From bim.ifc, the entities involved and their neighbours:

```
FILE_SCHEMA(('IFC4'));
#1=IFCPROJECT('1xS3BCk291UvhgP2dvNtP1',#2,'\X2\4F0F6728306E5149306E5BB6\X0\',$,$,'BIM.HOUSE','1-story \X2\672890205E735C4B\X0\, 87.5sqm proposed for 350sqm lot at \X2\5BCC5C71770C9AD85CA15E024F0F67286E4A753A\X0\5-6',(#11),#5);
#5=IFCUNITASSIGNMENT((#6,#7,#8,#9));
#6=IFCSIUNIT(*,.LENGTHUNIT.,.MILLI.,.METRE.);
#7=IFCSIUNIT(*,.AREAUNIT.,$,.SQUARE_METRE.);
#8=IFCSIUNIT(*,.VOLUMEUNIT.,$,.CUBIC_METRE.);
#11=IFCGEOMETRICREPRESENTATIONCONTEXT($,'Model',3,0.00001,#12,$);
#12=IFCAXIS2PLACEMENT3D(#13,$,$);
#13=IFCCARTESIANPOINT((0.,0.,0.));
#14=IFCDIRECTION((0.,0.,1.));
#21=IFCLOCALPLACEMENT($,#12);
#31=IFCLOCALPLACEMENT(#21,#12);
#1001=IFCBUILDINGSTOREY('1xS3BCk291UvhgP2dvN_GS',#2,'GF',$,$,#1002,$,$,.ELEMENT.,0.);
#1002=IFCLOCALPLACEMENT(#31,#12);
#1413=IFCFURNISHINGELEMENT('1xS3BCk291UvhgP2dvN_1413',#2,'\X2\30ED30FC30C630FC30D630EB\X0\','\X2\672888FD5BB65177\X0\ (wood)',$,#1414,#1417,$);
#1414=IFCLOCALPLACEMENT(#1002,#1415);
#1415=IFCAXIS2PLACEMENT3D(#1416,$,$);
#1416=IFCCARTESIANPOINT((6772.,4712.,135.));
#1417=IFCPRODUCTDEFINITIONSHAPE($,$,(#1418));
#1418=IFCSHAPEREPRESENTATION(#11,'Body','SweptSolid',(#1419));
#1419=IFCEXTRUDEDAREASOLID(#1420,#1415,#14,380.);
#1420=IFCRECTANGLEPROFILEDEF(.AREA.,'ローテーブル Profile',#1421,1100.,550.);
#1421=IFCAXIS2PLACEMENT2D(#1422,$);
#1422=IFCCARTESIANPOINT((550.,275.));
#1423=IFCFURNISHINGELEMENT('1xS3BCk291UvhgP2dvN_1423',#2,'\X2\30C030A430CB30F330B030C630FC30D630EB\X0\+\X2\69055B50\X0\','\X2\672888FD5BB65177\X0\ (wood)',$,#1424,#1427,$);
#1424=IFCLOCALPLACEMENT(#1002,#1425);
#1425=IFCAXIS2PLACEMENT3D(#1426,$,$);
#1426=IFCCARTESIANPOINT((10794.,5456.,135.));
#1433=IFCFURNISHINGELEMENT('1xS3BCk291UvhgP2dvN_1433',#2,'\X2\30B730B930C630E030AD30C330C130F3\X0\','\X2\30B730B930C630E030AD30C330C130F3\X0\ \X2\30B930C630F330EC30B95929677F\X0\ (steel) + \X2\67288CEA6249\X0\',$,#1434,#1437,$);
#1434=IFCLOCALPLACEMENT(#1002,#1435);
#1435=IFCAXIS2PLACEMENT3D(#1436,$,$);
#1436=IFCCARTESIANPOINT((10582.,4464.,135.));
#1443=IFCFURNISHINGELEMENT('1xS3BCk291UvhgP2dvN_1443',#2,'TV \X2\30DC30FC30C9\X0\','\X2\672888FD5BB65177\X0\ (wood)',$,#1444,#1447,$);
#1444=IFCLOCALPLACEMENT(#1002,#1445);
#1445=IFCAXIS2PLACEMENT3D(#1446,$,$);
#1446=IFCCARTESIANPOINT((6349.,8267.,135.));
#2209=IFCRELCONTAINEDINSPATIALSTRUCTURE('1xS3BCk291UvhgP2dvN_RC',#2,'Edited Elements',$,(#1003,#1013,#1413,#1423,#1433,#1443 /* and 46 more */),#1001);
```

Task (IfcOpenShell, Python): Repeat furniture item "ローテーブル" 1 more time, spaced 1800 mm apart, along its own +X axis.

```python
import ifcopenshell
import ifcopenshell.api.geometry
import ifcopenshell.api.root
import ifcopenshell.util.element
import ifcopenshell.util.placement
import ifcopenshell.util.unit

model = ifcopenshell.open("bim.ifc")
unit_scale = ifcopenshell.util.unit.calculate_unit_scale(model)


def reuse_history(source, copy):
    """copy_class also copies each property set's owner history, people and application; keep the originals."""
    for rel in copy.IsDefinedBy:
        if rel.is_a("IfcRelDefinesByProperties") and (history := rel.RelatingPropertyDefinition.OwnerHistory):
            rel.RelatingPropertyDefinition.OwnerHistory = source.OwnerHistory
            ifcopenshell.util.element.remove_deep2(model, history)


source = model.by_guid("1xS3BCk291UvhgP2dvN_1413")
base = ifcopenshell.util.placement.get_local_placement(source.ObjectPlacement)
step = base[:3, 0] * 1.8 / unit_scale

for i in range(1, 2):
    copy = ifcopenshell.api.root.copy_class(model, product=source)
    copy.Representation = ifcopenshell.util.element.copy_deep(
        model, source.Representation, exclude=["IfcGeometricRepresentationContext", "IfcRepresentationMap"]
    )
    reuse_history(source, copy)
    matrix = base.copy()
    matrix[:3, 3] += i * step
    print("added at", matrix[:3, 3].round(3) + 0.0)
    ifcopenshell.api.geometry.edit_object_placement(model, product=copy, matrix=matrix, is_si=False)

model.write("bim_updated.ifc")
```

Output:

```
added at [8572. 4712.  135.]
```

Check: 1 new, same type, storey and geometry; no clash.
